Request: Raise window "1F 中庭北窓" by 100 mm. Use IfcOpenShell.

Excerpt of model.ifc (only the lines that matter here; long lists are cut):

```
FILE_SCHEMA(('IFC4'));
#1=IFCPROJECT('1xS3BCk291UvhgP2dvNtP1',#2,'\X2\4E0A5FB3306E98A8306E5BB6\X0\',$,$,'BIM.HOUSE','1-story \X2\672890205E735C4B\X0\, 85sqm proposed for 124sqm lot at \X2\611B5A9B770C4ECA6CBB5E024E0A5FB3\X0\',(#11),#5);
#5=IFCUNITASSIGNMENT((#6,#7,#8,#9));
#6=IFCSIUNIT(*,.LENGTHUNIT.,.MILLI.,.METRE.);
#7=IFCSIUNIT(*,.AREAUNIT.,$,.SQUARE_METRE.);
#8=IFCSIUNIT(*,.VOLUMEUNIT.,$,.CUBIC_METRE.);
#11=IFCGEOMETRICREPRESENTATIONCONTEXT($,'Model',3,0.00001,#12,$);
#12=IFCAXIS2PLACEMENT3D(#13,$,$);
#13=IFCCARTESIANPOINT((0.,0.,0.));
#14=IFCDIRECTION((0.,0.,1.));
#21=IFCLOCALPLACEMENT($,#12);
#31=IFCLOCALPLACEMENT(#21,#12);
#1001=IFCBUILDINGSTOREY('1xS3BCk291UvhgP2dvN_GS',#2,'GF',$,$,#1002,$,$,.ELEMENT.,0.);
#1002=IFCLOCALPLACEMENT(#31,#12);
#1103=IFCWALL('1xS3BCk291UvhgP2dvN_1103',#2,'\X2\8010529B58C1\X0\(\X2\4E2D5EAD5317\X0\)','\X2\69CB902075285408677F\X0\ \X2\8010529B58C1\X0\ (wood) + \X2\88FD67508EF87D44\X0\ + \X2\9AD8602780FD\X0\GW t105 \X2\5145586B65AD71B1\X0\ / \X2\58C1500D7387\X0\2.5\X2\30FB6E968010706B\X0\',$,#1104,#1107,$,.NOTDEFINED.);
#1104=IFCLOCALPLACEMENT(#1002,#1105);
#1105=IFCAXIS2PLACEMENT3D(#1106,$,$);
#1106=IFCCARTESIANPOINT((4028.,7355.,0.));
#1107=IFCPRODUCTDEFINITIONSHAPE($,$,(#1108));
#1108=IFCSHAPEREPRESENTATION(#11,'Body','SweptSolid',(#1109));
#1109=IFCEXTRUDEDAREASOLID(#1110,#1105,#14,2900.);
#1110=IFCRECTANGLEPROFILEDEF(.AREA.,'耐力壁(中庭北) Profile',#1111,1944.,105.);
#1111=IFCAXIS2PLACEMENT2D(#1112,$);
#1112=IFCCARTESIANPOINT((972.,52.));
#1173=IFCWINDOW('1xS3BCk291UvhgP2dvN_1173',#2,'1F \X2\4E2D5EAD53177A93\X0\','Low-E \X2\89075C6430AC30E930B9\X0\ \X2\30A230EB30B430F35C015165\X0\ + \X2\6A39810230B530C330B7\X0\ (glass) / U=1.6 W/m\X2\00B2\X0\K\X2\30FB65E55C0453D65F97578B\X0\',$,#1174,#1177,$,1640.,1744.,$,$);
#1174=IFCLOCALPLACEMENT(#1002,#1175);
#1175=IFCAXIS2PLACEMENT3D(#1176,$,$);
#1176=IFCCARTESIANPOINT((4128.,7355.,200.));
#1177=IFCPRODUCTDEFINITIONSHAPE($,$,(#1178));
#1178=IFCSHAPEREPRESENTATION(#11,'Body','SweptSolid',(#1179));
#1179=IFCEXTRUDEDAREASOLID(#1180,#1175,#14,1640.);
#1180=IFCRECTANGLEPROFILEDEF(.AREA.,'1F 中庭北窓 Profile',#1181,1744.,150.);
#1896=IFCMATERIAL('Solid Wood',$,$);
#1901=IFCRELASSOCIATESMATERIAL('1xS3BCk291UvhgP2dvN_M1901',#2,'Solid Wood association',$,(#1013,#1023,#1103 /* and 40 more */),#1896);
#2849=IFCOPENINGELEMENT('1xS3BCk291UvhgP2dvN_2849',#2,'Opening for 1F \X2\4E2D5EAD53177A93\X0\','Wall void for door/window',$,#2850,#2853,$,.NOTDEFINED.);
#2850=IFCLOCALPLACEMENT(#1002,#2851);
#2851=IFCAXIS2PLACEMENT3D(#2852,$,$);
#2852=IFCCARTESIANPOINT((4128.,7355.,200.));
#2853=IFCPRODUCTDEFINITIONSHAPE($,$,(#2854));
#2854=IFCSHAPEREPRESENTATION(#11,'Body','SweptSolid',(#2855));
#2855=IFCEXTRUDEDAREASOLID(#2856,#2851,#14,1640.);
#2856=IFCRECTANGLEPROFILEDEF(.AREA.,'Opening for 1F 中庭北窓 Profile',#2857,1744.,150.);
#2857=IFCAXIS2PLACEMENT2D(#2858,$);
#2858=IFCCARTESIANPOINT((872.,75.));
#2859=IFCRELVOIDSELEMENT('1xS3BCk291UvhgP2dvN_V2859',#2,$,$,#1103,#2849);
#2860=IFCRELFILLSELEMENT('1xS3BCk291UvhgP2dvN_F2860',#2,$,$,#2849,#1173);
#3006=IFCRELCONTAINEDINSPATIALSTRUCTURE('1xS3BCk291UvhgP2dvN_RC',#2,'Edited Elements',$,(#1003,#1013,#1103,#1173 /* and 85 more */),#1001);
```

```python
import numpy as np
import ifcopenshell
import ifcopenshell.api.geometry
import ifcopenshell.util.placement
import ifcopenshell.util.unit

model = ifcopenshell.open("model.ifc")
unit_scale = ifcopenshell.util.unit.calculate_unit_scale(model)

window = model.by_guid("1xS3BCk291UvhgP2dvN_1173")
opening = window.FillsVoids[0].RelatingOpeningElement
dz = 0.1 / unit_scale

shift = np.array([0.0, 0.0, dz])
# The window is not placed relative to its opening, so move both.
for product in (opening, window):
    matrix = ifcopenshell.util.placement.get_local_placement(product.ObjectPlacement)
    matrix[:3, 3] += shift
    ifcopenshell.api.geometry.edit_object_placement(model, product=product, matrix=matrix, is_si=False)

print(f"moved by {dz * unit_scale:+.3f} m")

model.write("model_edited.ifc")
```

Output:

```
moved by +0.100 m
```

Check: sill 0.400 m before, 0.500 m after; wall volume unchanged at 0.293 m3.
